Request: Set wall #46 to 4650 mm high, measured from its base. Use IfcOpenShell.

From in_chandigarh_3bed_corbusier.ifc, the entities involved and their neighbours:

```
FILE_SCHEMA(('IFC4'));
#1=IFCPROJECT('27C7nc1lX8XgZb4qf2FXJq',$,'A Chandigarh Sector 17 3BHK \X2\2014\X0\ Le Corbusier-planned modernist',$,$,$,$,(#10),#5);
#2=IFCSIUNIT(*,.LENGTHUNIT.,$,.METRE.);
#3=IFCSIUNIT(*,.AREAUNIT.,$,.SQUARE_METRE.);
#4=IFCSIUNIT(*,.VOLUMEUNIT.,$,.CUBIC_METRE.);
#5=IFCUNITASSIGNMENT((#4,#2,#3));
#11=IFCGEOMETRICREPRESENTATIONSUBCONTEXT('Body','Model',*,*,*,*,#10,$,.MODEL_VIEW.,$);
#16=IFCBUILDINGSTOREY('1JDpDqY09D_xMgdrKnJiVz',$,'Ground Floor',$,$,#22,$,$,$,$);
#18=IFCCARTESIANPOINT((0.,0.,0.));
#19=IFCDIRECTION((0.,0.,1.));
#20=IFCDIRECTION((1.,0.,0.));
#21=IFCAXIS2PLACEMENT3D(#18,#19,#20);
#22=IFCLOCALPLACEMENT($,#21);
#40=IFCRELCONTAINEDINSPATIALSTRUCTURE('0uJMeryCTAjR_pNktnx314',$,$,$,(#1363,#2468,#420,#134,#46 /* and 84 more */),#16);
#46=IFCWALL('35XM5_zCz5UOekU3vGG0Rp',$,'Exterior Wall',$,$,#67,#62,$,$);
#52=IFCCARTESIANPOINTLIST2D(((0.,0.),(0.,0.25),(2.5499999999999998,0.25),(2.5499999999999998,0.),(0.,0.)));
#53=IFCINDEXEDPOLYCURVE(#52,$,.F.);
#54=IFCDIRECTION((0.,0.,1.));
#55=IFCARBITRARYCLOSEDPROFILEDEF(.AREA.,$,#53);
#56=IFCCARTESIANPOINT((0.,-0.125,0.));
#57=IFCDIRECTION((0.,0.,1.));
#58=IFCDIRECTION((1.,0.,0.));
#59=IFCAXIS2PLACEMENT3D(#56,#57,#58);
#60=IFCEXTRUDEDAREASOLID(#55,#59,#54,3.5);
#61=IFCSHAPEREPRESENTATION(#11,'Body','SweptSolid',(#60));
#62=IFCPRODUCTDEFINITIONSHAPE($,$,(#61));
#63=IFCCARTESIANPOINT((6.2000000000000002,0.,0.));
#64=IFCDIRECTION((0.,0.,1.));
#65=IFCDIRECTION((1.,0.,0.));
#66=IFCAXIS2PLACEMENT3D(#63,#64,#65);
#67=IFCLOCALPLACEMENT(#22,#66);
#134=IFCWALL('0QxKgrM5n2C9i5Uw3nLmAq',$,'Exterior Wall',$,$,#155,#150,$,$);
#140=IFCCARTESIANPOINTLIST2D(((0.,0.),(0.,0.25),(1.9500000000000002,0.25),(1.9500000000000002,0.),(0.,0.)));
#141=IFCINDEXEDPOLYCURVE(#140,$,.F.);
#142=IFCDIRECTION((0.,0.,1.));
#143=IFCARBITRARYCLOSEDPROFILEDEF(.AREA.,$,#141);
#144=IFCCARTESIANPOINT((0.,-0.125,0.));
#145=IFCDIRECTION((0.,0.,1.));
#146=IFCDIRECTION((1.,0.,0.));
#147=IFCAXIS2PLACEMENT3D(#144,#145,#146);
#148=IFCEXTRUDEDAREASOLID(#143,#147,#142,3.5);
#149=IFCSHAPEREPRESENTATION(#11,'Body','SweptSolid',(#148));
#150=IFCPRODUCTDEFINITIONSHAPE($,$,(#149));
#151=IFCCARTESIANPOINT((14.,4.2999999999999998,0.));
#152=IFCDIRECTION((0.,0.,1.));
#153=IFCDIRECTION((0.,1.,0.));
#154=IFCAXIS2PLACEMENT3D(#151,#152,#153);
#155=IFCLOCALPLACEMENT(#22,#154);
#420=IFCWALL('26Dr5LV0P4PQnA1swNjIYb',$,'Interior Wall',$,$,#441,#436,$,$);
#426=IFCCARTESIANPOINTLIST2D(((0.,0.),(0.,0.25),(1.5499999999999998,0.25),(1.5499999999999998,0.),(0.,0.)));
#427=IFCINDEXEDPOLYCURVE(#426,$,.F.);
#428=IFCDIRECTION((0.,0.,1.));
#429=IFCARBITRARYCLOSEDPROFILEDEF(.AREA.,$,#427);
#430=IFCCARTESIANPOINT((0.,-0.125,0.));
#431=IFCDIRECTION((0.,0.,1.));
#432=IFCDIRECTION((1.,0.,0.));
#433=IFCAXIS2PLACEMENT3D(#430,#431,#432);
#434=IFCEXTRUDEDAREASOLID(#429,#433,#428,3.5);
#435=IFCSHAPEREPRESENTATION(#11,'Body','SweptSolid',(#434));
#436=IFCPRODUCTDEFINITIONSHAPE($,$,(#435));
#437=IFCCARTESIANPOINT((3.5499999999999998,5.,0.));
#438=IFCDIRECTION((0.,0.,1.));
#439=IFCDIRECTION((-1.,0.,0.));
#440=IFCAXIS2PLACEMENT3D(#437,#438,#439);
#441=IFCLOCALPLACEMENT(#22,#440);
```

```python
import ifcopenshell
import ifcopenshell.geom
import ifcopenshell.util.representation
import ifcopenshell.util.shape
import ifcopenshell.util.unit

model = ifcopenshell.open("in_chandigarh_3bed_corbusier.ifc")
unit_scale = ifcopenshell.util.unit.calculate_unit_scale(model)
settings = ifcopenshell.geom.settings()


def volume(element):
    """Net volume in cubic metres, openings subtracted."""
    shape = ifcopenshell.geom.create_shape(settings, element)
    return ifcopenshell.util.shape.get_volume(shape.geometry)


wall = model.by_guid("35XM5_zCz5UOekU3vGG0Rp")
before = volume(wall)

body = ifcopenshell.util.representation.get_representation(wall, "Model", "Body")
solid = body.Items[0]
old_height = solid.Depth
solid.Depth = 4.65 / unit_scale
after = volume(wall)

print(f"height {old_height:g} -> {solid.Depth:g}, volume {before:.3f} -> {after:.3f} m3")

model.write("in_chandigarh_3bed_corbusier_updated.ifc")
```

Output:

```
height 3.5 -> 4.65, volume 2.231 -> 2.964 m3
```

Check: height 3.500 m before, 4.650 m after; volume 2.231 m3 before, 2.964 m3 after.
